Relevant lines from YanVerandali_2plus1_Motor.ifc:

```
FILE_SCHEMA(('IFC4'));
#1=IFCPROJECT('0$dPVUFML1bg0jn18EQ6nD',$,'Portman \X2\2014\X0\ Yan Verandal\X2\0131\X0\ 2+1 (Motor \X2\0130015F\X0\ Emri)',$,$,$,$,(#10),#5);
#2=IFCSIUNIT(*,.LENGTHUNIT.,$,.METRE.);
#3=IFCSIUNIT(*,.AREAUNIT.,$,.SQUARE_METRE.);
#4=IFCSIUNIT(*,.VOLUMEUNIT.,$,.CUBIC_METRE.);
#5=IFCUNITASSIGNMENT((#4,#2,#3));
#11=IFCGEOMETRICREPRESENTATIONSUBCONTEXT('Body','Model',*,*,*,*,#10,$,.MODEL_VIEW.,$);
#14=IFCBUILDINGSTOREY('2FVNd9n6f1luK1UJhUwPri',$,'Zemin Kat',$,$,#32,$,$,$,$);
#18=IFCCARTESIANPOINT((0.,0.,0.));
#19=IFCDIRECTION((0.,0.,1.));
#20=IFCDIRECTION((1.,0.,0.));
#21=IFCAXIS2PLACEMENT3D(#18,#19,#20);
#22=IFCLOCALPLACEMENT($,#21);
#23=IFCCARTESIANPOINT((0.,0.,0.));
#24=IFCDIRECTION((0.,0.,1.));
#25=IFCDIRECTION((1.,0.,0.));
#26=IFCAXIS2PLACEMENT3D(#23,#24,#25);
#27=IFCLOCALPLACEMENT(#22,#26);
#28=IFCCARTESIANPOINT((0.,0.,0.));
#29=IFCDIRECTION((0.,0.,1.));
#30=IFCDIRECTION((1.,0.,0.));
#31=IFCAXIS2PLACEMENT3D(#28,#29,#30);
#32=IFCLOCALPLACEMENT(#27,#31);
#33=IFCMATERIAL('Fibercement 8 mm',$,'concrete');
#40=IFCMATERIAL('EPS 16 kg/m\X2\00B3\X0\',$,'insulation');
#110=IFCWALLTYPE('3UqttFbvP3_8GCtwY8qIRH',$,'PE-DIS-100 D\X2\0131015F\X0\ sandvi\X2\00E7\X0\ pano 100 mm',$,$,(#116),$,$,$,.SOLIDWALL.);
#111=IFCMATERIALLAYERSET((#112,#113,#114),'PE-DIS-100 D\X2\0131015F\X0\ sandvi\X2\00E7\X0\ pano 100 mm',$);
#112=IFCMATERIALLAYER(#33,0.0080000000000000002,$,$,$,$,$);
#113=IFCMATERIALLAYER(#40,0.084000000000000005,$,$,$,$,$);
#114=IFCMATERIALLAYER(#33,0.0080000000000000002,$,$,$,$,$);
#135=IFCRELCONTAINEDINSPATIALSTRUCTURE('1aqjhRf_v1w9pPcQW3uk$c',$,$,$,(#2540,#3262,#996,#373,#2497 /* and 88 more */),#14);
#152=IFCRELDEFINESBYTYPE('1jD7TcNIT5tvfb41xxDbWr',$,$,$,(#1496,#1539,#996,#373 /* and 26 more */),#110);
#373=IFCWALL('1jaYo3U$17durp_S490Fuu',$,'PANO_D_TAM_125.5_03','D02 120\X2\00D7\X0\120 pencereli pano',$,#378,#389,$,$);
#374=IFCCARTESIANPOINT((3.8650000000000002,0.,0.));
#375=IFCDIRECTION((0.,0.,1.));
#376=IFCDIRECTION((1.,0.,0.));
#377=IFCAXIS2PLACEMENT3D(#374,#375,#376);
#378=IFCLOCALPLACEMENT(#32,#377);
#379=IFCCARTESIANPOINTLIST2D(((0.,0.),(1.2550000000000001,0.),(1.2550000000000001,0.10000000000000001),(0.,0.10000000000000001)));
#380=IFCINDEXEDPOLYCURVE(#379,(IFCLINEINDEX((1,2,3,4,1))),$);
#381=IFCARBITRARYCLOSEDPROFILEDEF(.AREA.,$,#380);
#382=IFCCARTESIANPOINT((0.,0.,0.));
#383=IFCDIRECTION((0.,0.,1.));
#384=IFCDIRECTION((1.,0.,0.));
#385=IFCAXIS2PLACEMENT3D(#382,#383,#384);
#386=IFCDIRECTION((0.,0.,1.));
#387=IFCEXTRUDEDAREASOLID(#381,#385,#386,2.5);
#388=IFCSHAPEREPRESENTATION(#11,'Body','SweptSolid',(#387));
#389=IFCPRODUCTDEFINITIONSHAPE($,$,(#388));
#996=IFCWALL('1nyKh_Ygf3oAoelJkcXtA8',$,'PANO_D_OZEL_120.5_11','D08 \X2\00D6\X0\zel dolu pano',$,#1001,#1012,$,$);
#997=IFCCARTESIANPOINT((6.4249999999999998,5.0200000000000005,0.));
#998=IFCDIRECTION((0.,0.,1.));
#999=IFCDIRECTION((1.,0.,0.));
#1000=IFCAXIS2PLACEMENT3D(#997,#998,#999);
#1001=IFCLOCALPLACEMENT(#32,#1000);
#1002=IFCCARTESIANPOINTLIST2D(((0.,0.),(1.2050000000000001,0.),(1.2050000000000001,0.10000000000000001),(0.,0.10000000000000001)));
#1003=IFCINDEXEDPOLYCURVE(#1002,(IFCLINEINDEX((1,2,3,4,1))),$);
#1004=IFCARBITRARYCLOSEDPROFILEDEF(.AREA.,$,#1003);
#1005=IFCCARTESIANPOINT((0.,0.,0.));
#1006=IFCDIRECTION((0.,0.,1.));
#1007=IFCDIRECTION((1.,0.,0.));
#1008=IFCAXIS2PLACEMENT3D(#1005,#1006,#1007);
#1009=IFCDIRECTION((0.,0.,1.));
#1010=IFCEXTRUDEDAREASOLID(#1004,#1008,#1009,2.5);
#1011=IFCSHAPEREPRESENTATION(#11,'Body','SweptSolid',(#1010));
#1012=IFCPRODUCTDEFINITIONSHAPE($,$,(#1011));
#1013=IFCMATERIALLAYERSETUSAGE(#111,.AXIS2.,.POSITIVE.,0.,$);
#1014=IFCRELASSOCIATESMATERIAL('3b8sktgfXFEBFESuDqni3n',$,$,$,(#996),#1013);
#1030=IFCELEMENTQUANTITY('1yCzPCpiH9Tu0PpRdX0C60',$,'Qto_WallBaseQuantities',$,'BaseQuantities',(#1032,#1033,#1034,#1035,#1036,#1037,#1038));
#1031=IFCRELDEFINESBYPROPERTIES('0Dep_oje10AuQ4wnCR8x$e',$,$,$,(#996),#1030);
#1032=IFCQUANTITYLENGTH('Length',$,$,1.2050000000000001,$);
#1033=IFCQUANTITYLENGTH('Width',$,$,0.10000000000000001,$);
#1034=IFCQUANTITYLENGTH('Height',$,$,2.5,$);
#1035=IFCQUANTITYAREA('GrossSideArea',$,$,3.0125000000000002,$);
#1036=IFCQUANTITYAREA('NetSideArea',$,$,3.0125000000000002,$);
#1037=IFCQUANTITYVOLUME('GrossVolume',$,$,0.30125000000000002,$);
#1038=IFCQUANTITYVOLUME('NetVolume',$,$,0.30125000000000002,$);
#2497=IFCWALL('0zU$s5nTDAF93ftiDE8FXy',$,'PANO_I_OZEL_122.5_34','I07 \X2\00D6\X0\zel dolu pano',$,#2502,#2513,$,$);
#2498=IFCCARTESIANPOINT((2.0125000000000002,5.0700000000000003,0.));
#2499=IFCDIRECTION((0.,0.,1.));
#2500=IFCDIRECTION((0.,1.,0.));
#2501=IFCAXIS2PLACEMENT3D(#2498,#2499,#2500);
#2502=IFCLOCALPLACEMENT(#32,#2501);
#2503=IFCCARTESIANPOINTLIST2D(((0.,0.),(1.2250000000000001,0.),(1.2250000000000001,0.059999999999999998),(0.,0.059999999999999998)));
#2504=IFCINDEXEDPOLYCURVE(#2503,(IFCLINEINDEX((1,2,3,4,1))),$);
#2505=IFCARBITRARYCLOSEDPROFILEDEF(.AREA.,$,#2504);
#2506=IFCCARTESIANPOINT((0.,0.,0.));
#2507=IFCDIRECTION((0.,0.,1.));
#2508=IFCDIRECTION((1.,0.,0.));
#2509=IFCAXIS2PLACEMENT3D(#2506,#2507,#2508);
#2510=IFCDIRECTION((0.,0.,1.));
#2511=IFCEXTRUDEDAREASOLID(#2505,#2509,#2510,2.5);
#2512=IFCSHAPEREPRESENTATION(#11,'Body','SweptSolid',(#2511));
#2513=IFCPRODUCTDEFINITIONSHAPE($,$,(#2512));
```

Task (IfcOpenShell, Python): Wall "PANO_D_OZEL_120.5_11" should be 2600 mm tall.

```python
import ifcopenshell
import ifcopenshell.api.pset
import ifcopenshell.geom
import ifcopenshell.util.element
import ifcopenshell.util.representation
import ifcopenshell.util.shape
import ifcopenshell.util.unit

model = ifcopenshell.open("YanVerandali_2plus1_Motor.ifc")
unit_scale = ifcopenshell.util.unit.calculate_unit_scale(model)
area_scale = ifcopenshell.util.unit.calculate_unit_scale(model, "AREAUNIT")
volume_scale = ifcopenshell.util.unit.calculate_unit_scale(model, "VOLUMEUNIT")
settings = ifcopenshell.geom.settings()


def volume(element):
    """Net volume in cubic metres, openings subtracted."""
    shape = ifcopenshell.geom.create_shape(settings, element)
    return ifcopenshell.util.shape.get_volume(shape.geometry)


wall = model.by_guid("1nyKh_Ygf3oAoelJkcXtA8")
before = volume(wall)

body = ifcopenshell.util.representation.get_representation(wall, "Model", "Body")
solid = body.Items[0]
old_height = solid.Depth
solid.Depth = 2.6 / unit_scale
after = volume(wall)
thickness = 0.1  # wall thickness in metres

# Update the stored height, areas and volumes.
qto = model.by_id(ifcopenshell.util.element.get_pset(wall, "Qto_WallBaseQuantities", should_inherit=False)["id"])
ifcopenshell.api.pset.edit_qto(model, qto=qto, properties={
    "Height": solid.Depth,
    "GrossSideArea": ifcopenshell.util.element.get_pset(wall, "Qto_WallBaseQuantities", "GrossSideArea") * solid.Depth / old_height,
    "NetSideArea": after / thickness / area_scale,
    "GrossVolume": ifcopenshell.util.element.get_pset(wall, "Qto_WallBaseQuantities", "GrossVolume") * solid.Depth / old_height,
    "NetVolume": after / volume_scale,
})

print(f"height {old_height:g} -> {solid.Depth:g}, volume {before:.3f} -> {after:.3f} m3")

model.write("YanVerandali_2plus1_Motor_rev.ifc")
```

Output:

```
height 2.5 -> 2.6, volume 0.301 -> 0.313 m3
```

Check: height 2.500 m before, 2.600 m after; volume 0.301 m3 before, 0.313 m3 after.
